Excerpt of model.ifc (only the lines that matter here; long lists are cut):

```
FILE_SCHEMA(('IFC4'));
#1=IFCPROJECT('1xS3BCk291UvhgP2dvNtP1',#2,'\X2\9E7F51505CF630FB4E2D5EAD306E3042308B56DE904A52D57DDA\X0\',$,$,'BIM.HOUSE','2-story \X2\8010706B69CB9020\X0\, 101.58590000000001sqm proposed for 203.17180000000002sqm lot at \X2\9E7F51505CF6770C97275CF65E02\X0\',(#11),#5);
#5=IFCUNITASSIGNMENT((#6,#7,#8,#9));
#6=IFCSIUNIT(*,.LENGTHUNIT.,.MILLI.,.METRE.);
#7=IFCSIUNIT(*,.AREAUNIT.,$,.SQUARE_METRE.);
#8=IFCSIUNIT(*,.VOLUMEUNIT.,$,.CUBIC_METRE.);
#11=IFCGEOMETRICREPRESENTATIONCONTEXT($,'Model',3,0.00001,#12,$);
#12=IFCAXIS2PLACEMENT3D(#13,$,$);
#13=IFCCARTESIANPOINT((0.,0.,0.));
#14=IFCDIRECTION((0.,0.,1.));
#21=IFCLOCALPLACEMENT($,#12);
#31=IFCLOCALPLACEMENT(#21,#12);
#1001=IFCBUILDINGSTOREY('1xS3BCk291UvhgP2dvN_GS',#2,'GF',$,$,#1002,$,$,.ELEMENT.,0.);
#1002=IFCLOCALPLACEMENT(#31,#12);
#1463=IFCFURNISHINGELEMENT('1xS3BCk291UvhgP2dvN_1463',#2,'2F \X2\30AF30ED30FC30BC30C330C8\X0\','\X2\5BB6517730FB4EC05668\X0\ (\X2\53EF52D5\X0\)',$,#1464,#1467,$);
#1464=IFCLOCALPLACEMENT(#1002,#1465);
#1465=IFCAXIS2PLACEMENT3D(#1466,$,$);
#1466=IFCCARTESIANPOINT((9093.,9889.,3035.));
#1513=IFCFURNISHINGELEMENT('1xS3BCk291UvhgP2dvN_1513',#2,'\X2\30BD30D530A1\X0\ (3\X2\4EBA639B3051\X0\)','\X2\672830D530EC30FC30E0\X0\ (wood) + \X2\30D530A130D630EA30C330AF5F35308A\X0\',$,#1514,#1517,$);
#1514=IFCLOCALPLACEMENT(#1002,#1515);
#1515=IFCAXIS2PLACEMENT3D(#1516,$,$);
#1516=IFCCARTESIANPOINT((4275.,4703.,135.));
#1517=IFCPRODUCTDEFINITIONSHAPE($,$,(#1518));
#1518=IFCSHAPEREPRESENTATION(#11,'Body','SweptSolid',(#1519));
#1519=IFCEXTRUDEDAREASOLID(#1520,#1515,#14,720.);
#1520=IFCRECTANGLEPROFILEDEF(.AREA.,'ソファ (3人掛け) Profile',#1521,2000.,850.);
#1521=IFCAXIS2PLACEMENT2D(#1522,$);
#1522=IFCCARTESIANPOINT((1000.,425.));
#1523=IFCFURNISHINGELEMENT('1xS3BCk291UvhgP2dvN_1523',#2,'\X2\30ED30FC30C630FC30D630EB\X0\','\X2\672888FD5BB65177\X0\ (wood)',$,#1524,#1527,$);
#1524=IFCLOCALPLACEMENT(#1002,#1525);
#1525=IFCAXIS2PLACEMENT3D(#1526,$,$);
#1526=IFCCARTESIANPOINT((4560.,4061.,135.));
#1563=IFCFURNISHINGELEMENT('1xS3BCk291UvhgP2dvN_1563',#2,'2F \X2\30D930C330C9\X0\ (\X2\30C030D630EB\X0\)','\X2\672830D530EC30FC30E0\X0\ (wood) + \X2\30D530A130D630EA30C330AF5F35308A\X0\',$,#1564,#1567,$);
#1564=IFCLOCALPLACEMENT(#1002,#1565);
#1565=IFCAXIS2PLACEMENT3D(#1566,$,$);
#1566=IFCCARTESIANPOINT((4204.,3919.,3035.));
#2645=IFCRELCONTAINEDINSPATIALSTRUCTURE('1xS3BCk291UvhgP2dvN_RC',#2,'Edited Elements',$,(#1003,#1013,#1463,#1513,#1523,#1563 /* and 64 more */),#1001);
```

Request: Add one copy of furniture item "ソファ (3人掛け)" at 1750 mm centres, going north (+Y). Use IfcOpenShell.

```python
import numpy as np
import ifcopenshell
import ifcopenshell.api.geometry
import ifcopenshell.api.root
import ifcopenshell.util.element
import ifcopenshell.util.placement
import ifcopenshell.util.unit

model = ifcopenshell.open("model.ifc")
unit_scale = ifcopenshell.util.unit.calculate_unit_scale(model)


def reuse_history(source, copy):
    """copy_class also copies each property set's owner history, people and application; keep the originals."""
    for rel in copy.IsDefinedBy:
        if rel.is_a("IfcRelDefinesByProperties") and (history := rel.RelatingPropertyDefinition.OwnerHistory):
            rel.RelatingPropertyDefinition.OwnerHistory = source.OwnerHistory
            ifcopenshell.util.element.remove_deep2(model, history)


source = model.by_id(1513)
base = ifcopenshell.util.placement.get_local_placement(source.ObjectPlacement)
step = np.array([0.0, 1.0, 0.0]) * 1.75 / unit_scale

for i in range(1, 2):
    copy = ifcopenshell.api.root.copy_class(model, product=source)
    copy.Representation = ifcopenshell.util.element.copy_deep(
        model, source.Representation, exclude=["IfcGeometricRepresentationContext", "IfcRepresentationMap"]
    )
    reuse_history(source, copy)
    matrix = base.copy()
    matrix[:3, 3] += i * step
    print("added at", matrix[:3, 3].round(3) + 0.0)
    ifcopenshell.api.geometry.edit_object_placement(model, product=copy, matrix=matrix, is_si=False)

model.write("model_updated.ifc")
```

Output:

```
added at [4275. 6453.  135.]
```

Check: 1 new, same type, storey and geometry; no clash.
